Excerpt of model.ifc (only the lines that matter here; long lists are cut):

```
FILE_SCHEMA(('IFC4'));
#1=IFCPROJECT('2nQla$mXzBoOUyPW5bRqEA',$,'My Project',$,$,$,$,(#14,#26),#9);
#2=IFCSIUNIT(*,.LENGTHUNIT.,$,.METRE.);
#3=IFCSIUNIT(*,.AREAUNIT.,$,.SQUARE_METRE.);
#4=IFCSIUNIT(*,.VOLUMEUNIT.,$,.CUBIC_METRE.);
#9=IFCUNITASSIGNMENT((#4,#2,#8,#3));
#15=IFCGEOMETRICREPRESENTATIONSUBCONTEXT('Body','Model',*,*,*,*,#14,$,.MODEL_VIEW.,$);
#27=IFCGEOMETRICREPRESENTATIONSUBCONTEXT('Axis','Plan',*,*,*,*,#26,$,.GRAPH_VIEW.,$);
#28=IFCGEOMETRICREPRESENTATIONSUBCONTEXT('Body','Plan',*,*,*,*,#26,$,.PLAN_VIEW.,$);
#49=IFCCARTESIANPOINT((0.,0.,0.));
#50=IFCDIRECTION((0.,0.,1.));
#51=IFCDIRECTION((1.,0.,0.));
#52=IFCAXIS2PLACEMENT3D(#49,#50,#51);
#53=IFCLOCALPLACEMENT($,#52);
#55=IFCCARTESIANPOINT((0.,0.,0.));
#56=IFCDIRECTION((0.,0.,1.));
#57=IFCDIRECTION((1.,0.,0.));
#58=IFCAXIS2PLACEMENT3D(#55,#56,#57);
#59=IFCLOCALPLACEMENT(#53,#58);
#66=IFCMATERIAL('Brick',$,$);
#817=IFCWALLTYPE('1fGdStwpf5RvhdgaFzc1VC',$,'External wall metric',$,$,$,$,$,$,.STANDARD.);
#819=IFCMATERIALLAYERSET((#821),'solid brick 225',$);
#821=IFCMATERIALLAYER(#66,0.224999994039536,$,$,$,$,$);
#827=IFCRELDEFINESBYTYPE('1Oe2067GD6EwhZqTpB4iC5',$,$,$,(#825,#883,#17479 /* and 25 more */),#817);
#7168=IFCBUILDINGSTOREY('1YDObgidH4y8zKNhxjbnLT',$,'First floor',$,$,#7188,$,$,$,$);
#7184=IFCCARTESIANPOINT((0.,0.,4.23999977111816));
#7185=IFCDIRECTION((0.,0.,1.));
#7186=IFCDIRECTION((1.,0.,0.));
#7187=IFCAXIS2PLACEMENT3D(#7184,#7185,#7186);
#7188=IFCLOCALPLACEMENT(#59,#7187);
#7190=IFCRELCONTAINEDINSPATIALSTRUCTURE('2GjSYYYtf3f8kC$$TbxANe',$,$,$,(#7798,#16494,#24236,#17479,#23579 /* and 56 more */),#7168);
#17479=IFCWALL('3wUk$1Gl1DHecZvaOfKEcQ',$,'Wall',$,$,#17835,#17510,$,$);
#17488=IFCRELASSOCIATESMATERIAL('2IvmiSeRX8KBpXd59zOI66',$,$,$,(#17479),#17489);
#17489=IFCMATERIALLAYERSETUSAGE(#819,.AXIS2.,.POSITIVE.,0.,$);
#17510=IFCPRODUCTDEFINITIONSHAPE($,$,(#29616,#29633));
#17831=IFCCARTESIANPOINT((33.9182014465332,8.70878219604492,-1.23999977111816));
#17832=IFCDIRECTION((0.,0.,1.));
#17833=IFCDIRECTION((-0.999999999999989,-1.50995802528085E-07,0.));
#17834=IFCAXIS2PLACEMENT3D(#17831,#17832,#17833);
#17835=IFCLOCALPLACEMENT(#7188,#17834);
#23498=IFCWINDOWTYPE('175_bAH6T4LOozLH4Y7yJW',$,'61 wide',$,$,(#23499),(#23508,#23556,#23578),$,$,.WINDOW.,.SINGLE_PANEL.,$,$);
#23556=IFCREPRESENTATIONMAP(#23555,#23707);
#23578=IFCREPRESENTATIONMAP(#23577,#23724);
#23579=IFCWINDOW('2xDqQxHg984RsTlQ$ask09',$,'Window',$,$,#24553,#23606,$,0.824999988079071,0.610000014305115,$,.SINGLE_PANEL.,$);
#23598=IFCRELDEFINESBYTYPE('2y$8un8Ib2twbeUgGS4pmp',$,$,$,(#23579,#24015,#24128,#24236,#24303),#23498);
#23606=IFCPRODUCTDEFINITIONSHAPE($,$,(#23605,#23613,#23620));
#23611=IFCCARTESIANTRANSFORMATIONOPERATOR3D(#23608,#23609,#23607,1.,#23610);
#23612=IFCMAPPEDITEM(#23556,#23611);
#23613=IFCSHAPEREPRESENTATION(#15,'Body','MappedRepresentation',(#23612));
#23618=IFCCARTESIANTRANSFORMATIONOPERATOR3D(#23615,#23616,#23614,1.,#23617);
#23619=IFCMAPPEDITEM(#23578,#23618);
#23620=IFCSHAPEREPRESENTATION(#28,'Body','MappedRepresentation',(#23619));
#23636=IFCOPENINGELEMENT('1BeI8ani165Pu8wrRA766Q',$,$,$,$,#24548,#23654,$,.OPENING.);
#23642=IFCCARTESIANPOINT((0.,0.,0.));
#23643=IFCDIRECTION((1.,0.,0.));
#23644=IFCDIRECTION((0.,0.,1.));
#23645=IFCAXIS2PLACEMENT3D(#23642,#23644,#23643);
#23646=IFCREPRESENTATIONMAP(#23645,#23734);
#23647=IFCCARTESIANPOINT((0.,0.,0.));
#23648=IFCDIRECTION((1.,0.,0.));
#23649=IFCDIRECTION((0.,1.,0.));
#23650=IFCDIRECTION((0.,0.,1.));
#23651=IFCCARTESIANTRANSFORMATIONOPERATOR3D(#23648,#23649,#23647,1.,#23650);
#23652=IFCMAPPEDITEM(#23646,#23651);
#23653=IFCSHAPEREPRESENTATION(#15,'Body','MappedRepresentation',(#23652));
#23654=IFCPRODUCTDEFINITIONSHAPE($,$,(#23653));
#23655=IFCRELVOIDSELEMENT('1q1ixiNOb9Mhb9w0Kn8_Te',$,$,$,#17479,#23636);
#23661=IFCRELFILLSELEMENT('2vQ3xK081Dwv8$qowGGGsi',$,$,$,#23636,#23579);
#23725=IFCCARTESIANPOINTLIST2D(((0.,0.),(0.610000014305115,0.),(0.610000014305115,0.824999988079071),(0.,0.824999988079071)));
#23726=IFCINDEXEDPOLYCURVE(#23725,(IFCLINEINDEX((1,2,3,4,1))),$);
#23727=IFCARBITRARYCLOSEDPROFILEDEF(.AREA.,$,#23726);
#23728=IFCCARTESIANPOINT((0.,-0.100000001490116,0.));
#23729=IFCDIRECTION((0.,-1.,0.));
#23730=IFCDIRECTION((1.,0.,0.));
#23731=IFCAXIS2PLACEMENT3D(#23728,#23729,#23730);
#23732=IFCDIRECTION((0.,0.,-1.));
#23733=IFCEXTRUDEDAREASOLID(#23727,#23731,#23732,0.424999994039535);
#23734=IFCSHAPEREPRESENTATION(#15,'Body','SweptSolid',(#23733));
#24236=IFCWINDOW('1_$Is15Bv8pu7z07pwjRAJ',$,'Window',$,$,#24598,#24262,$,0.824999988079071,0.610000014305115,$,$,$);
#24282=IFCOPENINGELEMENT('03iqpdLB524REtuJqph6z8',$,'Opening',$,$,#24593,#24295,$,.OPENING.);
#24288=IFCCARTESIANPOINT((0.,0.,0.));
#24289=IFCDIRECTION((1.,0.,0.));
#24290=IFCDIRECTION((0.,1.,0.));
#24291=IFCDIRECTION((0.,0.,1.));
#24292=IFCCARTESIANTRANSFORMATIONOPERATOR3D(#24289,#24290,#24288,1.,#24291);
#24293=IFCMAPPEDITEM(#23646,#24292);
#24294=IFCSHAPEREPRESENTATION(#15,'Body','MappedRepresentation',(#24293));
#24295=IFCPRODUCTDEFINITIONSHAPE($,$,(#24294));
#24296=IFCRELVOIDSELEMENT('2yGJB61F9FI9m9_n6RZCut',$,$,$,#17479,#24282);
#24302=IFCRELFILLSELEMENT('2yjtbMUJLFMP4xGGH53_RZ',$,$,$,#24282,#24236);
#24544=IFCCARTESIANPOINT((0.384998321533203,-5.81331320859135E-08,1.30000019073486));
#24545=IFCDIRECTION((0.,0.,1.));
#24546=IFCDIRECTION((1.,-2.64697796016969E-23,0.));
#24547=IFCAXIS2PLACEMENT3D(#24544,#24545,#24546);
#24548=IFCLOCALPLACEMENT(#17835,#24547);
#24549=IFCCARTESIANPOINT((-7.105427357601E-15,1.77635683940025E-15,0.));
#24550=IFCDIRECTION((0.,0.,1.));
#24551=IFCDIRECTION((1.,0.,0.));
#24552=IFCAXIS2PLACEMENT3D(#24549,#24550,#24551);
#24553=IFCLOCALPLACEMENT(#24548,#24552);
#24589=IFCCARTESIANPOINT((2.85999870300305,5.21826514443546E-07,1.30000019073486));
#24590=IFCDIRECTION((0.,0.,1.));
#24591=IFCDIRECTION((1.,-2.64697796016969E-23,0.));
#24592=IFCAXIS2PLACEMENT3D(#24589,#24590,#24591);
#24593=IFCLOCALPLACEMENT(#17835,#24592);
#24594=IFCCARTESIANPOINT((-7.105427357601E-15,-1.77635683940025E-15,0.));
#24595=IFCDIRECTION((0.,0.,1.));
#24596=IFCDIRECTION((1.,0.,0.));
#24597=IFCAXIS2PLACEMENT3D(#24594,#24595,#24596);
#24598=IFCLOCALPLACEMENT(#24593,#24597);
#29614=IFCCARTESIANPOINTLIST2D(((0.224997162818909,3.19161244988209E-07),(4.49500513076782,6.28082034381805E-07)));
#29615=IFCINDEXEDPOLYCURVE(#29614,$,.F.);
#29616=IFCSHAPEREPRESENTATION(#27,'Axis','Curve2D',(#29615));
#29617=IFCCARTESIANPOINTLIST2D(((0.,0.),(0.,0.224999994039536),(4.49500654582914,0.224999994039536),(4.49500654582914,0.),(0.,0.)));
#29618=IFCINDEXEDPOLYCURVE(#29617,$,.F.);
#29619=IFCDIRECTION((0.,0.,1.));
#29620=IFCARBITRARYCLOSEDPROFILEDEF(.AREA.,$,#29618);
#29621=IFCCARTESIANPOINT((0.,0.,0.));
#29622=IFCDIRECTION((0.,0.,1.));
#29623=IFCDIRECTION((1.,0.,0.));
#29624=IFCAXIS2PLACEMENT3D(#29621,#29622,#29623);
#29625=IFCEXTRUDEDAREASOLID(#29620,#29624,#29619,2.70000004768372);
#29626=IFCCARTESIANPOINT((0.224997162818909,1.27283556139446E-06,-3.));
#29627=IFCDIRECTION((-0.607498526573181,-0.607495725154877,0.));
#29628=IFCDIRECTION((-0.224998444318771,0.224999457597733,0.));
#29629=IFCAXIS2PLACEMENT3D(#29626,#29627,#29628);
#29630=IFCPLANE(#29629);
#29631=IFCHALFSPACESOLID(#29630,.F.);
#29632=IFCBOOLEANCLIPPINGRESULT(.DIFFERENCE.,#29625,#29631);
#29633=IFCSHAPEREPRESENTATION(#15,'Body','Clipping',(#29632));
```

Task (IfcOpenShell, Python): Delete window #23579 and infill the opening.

```python
import ifcopenshell
import ifcopenshell.api.feature
import ifcopenshell.api.root
import ifcopenshell.geom
import ifcopenshell.util.shape

model = ifcopenshell.open("model.ifc")
settings = ifcopenshell.geom.settings()


def volume(element):
    """Net volume in cubic metres, openings subtracted."""
    shape = ifcopenshell.geom.create_shape(settings, element)
    return ifcopenshell.util.shape.get_volume(shape.geometry)


window = model.by_id(23579)
opening = window.FillsVoids[0].RelatingOpeningElement
wall = opening.VoidsElements[0].RelatingBuildingElement
before = volume(wall)

ifcopenshell.api.root.remove_product(model, product=window)
ifcopenshell.api.feature.remove_feature(model, feature=opening)

after = volume(wall)

print(f"wall volume {before:.3f} -> {after:.3f} m3")

model.write("model-out.ifc")
```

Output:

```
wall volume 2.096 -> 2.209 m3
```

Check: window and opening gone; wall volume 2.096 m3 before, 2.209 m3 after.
